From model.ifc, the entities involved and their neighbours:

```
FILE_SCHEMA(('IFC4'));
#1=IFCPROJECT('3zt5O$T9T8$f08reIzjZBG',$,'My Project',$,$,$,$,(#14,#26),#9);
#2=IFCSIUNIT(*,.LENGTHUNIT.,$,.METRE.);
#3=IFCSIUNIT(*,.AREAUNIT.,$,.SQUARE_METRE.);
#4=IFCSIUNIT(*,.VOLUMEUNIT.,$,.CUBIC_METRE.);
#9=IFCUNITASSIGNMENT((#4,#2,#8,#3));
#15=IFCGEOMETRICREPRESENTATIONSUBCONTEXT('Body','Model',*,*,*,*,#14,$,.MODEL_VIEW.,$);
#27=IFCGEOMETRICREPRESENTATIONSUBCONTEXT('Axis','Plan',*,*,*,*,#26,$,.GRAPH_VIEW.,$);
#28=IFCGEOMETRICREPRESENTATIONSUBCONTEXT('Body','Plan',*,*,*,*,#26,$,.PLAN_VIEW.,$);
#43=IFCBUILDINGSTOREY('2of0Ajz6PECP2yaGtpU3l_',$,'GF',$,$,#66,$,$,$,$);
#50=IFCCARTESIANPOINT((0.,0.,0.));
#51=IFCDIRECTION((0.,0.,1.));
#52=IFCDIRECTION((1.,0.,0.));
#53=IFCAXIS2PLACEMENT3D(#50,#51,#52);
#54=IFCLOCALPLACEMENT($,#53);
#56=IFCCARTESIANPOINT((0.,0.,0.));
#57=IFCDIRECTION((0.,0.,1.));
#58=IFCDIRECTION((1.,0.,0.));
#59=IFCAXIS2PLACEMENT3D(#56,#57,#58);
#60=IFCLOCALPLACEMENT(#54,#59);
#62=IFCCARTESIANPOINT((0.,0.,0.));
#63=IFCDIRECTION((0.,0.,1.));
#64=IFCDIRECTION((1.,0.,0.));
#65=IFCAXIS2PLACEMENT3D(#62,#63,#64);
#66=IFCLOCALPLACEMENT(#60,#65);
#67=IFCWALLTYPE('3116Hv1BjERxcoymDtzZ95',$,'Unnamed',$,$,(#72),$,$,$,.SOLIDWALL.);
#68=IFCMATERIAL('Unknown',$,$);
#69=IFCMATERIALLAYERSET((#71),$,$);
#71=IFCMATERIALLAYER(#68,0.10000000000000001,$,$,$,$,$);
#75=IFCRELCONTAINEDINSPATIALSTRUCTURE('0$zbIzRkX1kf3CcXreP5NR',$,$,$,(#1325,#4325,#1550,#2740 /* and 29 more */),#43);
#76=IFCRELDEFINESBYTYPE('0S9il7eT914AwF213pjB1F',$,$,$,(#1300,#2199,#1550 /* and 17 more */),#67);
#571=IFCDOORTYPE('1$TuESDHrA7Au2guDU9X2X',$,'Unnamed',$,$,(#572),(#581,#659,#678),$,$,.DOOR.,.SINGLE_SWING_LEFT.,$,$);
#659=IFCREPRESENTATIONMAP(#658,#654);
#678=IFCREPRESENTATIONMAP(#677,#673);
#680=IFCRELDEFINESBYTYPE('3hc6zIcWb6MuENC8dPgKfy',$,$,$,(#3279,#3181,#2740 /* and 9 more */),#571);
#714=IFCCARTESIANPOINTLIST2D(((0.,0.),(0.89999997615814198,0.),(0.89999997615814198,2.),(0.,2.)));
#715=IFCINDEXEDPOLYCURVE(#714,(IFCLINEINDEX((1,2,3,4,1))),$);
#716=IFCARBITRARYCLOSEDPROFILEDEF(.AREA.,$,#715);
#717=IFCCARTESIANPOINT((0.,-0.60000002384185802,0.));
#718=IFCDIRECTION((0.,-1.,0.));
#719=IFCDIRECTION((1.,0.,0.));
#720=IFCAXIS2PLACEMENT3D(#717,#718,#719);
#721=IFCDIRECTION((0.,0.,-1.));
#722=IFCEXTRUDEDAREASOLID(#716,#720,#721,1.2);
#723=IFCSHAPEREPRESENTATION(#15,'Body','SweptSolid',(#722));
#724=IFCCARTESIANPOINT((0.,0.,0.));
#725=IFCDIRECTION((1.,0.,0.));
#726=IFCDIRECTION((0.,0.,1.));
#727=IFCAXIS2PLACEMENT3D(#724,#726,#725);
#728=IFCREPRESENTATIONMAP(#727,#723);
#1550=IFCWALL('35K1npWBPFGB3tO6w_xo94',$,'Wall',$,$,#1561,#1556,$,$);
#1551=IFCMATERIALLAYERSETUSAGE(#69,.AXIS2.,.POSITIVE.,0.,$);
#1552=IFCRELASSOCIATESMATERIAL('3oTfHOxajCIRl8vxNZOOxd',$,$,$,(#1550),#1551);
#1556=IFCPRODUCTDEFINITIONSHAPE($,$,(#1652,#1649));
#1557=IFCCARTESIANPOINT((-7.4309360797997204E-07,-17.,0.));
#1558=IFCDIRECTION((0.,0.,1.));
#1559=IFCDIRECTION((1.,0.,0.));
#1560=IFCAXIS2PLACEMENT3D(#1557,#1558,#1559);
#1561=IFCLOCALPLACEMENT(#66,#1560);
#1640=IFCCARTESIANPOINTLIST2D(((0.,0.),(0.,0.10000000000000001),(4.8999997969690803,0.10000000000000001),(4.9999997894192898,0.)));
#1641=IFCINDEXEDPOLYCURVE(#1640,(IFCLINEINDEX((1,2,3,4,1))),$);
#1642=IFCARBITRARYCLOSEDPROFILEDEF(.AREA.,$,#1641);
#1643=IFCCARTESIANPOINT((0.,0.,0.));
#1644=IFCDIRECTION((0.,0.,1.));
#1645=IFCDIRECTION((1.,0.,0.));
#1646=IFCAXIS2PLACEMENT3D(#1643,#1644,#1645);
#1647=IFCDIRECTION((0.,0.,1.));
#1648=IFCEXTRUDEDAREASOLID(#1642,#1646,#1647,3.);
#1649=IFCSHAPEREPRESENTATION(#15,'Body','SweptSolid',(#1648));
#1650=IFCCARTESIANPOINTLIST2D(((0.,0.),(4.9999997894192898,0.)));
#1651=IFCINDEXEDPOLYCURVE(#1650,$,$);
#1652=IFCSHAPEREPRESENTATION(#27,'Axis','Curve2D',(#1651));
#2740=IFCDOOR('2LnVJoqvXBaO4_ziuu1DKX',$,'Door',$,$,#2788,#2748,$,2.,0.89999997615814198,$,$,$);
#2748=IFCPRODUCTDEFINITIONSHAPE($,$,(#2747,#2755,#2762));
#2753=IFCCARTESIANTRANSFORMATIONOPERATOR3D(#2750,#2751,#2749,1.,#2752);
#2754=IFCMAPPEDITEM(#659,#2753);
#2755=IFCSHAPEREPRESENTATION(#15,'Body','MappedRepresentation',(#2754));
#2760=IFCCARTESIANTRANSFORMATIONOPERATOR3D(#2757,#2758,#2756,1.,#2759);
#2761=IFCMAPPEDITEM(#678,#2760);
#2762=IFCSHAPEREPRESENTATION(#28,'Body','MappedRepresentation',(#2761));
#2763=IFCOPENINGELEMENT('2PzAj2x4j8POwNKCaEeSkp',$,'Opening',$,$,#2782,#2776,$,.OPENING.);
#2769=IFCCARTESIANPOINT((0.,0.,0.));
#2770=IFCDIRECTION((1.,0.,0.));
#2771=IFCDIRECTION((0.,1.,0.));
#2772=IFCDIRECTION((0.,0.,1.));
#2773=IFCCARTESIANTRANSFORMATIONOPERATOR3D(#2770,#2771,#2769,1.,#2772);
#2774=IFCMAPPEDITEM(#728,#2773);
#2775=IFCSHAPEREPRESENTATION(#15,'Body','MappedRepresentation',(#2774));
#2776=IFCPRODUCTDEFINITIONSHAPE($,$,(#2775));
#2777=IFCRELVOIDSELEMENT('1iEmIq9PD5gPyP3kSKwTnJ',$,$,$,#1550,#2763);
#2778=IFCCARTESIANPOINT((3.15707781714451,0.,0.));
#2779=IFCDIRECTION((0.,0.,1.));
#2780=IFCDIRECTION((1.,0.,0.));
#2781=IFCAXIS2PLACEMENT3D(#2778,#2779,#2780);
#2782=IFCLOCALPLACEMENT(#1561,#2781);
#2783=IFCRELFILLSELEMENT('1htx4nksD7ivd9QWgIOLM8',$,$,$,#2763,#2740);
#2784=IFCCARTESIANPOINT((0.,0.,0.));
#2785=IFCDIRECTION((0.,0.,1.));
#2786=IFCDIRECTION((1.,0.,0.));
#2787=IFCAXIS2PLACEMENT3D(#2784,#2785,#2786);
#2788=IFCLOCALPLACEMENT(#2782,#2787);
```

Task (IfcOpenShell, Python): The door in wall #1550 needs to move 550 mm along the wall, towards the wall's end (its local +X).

```python
import ifcopenshell
import ifcopenshell.api.geometry
import ifcopenshell.util.placement

model = ifcopenshell.open("model.ifc")

door = model.by_guid("2LnVJoqvXBaO4_ziuu1DKX")
opening = door.FillsVoids[0].RelatingOpeningElement
wall = opening.VoidsElements[0].RelatingBuildingElement

wall_matrix = ifcopenshell.util.placement.get_local_placement(wall.ObjectPlacement)
shift = wall_matrix[:3, 0] * 0.55
before = ifcopenshell.util.placement.get_local_placement(door.ObjectPlacement)[:3, 3].copy()

# The door is placed relative to its opening, so it follows when the opening moves.
matrix = ifcopenshell.util.placement.get_local_placement(opening.ObjectPlacement)
matrix[:3, 3] += shift
ifcopenshell.api.geometry.edit_object_placement(
    model, product=opening, matrix=matrix, is_si=False, should_transform_children=True
)

after = ifcopenshell.util.placement.get_local_placement(door.ObjectPlacement)[:3, 3]
print("door moved by", (after - before).round(3) + 0.0)

model.write("model-out.ifc")
```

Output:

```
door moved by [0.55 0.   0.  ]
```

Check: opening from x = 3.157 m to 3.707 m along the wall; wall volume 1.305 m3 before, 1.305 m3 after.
